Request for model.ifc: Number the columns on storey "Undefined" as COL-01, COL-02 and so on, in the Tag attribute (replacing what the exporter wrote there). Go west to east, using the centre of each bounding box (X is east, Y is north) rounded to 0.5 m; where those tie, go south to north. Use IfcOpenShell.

First a look at what the model holds.

```python
import ifcopenshell
import ifcopenshell.util.element
import ifcopenshell.util.placement

model = ifcopenshell.open("model.ifc")
print(model.schema)
storey = next(s for s in model.by_type("IfcBuildingStorey") if s.Name == "Undefined")
columns = [e for e in ifcopenshell.util.element.get_decomposition(storey) if e.is_a("IfcColumn")]
for e in sorted(columns, key=lambda e: e.id()):
    origin = ifcopenshell.util.placement.get_local_placement(e.ObjectPlacement)[:3, 3]
    print(e.id(), e.Tag, e.Name, origin.round(2) + 0.0, sep=" | ")
```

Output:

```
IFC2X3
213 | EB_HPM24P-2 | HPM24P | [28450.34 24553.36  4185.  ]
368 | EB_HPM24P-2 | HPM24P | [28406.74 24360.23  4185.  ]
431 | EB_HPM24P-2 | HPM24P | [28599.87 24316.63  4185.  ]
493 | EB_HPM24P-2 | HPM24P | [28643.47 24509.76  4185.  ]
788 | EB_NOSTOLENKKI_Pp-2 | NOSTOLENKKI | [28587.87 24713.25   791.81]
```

```python
import ifcopenshell
import ifcopenshell.geom
import ifcopenshell.util.element
import ifcopenshell.util.shape

model = ifcopenshell.open("model.ifc")
settings = ifcopenshell.geom.settings()
settings.set("use-world-coords", True)


def centre(element):
    shape = ifcopenshell.geom.create_shape(settings, element)
    return ifcopenshell.util.shape.get_bbox_centroid(shape.geometry)


storey = next(s for s in model.by_type("IfcBuildingStorey") if s.Name == "Undefined")
columns = [e for e in ifcopenshell.util.element.get_decomposition(storey) if e.is_a("IfcColumn")]

# Insertion points can sit at a corner or the storey origin, so sort by the geometry (in metres).
centres = {e: centre(e) for e in columns}
columns.sort(key=lambda e: (round(centres[e][0] / 0.5), centres[e][1]))

for i, e in enumerate(columns, start=1):
    number = f"COL-{i:02d}"
    e.Tag = number
    print(e.id(), number)

model.write("model_rev.ifc")
```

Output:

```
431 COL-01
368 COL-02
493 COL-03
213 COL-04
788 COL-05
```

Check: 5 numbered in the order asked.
